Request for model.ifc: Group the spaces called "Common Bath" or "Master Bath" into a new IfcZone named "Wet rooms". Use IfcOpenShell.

First a look at what the model holds.

```python
import ifcopenshell

model = ifcopenshell.open("model.ifc")
print(model.schema)
seen = {}
for space in model.by_type("IfcSpace"):
    seen[space.LongName] = seen.get(space.LongName, 0) + 1
for name, count in sorted(seen.items(), key=str):
    print(count, "x", name)
print("zones:", [z.Name for z in model.by_type("IfcZone")][:20])
```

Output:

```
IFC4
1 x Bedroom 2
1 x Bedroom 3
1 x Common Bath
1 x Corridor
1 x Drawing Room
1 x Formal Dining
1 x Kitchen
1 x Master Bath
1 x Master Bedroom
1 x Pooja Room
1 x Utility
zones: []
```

```python
import ifcopenshell
import ifcopenshell.api.group
import ifcopenshell.api.root

model = ifcopenshell.open("model.ifc")

names = {"Common Bath", "Master Bath"}
spaces = [s for s in model.by_type("IfcSpace") if s.LongName in names]

zone = ifcopenshell.api.root.create_entity(model, ifc_class="IfcZone", name="Wet rooms")
ifcopenshell.api.group.assign_group(model, products=spaces, group=zone)
print(len(spaces), "spaces in", zone.Name)

model.write("model_rev.ifc")
```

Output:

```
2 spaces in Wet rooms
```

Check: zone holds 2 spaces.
